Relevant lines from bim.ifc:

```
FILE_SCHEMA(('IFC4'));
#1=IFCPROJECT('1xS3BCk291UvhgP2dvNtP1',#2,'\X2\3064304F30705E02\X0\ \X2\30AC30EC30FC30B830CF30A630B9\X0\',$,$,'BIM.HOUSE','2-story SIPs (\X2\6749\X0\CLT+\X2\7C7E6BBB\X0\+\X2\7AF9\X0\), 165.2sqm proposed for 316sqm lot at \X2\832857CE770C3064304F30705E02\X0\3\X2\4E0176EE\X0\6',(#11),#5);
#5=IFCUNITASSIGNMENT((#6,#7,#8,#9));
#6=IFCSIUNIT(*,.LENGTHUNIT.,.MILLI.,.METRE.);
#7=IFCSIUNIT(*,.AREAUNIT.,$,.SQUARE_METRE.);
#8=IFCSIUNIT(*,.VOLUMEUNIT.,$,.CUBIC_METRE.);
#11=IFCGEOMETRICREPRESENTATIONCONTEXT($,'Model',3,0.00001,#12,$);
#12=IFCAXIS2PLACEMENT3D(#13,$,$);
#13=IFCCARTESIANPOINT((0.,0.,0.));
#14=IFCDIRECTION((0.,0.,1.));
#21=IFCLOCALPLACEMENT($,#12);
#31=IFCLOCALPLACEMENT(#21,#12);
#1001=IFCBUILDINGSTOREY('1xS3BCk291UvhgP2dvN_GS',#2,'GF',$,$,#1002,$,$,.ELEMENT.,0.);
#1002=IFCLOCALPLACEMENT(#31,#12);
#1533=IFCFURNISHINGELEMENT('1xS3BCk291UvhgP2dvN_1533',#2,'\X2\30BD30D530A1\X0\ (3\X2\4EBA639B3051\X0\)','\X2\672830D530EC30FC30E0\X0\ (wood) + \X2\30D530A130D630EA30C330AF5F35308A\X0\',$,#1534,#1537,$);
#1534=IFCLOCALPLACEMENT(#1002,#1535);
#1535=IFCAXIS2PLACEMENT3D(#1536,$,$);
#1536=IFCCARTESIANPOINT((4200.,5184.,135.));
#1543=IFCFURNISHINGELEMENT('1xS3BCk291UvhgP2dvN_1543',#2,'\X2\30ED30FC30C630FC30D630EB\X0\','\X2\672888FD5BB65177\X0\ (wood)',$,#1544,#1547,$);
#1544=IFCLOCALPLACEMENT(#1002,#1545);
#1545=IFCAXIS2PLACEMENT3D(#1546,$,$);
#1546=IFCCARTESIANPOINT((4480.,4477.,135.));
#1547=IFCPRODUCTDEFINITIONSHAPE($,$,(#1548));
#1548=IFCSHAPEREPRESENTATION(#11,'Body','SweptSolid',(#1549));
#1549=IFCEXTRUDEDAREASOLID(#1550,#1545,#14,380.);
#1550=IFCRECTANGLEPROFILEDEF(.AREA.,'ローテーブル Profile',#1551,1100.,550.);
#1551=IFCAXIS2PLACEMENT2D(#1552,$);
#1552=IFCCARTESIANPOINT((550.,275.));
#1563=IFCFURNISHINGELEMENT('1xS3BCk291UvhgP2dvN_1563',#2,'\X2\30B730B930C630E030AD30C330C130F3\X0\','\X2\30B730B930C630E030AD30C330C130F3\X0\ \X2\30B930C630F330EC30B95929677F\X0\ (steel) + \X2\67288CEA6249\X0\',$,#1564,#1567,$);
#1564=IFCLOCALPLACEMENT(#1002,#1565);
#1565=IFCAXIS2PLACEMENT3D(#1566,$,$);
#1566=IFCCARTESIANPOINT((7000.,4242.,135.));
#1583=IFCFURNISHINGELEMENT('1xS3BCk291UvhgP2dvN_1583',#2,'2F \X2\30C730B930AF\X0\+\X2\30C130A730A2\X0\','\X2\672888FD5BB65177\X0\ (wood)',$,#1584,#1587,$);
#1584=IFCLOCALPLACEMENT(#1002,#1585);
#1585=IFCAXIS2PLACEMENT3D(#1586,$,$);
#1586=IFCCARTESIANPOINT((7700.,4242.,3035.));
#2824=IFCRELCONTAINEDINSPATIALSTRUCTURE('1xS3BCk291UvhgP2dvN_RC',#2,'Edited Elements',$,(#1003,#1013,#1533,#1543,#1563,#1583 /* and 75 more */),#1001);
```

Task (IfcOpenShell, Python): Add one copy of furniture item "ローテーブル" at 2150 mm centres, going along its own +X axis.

```python
import ifcopenshell
import ifcopenshell.api.geometry
import ifcopenshell.api.root
import ifcopenshell.util.element
import ifcopenshell.util.placement

model = ifcopenshell.open("bim.ifc")


def reuse_history(source, copy):
    """copy_class also copies each property set's owner history, people and application; keep the originals."""
    for rel in copy.IsDefinedBy:
        if rel.is_a("IfcRelDefinesByProperties") and (history := rel.RelatingPropertyDefinition.OwnerHistory):
            rel.RelatingPropertyDefinition.OwnerHistory = source.OwnerHistory
            ifcopenshell.util.element.remove_deep2(model, history)


source = model.by_guid("1xS3BCk291UvhgP2dvN_1543")
base = ifcopenshell.util.placement.get_local_placement(source.ObjectPlacement)
step = base[:3, 0] * 2150.0

for i in range(1, 2):
    copy = ifcopenshell.api.root.copy_class(model, product=source)
    copy.Representation = ifcopenshell.util.element.copy_deep(
        model, source.Representation, exclude=["IfcGeometricRepresentationContext", "IfcRepresentationMap"]
    )
    reuse_history(source, copy)
    matrix = base.copy()
    matrix[:3, 3] += i * step
    print("added at", matrix[:3, 3].round(3) + 0.0)
    ifcopenshell.api.geometry.edit_object_placement(model, product=copy, matrix=matrix, is_si=False)

model.write("bim-out.ifc")
```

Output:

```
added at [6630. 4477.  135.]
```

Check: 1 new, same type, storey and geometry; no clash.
